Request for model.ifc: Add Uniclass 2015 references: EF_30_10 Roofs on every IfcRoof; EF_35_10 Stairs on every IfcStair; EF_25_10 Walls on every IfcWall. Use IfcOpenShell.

First a look at what the model holds.

```python
import ifcopenshell

model = ifcopenshell.open("model.ifc")
print(model.schema)
print("classifications:", [c.Name for c in model.by_type("IfcClassification")])
for ifc_class in ("IfcDoor", "IfcRoof", "IfcStair", "IfcWall", "IfcWindow"):
    print(ifc_class, len(model.by_type(ifc_class)))
```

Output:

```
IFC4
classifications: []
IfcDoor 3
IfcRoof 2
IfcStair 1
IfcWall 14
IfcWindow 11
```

```python
import ifcopenshell
import ifcopenshell.api.classification

model = ifcopenshell.open("model.ifc")

system = ifcopenshell.api.classification.add_classification(model, classification="Uniclass 2015")

codes = {
    "IfcRoof": ("EF_30_10", "Roofs"),
    "IfcStair": ("EF_35_10", "Stairs"),
    "IfcWall": ("EF_25_10", "Walls"),
}
for ifc_class, (code, name) in codes.items():
    products = model.by_type(ifc_class)
    ifcopenshell.api.classification.add_reference(
        model, products=products, classification=system, identification=code, name=name
    )
    print(code, len(products))

model.write("model_rev.ifc")
```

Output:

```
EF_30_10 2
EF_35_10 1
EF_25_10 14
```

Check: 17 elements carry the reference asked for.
